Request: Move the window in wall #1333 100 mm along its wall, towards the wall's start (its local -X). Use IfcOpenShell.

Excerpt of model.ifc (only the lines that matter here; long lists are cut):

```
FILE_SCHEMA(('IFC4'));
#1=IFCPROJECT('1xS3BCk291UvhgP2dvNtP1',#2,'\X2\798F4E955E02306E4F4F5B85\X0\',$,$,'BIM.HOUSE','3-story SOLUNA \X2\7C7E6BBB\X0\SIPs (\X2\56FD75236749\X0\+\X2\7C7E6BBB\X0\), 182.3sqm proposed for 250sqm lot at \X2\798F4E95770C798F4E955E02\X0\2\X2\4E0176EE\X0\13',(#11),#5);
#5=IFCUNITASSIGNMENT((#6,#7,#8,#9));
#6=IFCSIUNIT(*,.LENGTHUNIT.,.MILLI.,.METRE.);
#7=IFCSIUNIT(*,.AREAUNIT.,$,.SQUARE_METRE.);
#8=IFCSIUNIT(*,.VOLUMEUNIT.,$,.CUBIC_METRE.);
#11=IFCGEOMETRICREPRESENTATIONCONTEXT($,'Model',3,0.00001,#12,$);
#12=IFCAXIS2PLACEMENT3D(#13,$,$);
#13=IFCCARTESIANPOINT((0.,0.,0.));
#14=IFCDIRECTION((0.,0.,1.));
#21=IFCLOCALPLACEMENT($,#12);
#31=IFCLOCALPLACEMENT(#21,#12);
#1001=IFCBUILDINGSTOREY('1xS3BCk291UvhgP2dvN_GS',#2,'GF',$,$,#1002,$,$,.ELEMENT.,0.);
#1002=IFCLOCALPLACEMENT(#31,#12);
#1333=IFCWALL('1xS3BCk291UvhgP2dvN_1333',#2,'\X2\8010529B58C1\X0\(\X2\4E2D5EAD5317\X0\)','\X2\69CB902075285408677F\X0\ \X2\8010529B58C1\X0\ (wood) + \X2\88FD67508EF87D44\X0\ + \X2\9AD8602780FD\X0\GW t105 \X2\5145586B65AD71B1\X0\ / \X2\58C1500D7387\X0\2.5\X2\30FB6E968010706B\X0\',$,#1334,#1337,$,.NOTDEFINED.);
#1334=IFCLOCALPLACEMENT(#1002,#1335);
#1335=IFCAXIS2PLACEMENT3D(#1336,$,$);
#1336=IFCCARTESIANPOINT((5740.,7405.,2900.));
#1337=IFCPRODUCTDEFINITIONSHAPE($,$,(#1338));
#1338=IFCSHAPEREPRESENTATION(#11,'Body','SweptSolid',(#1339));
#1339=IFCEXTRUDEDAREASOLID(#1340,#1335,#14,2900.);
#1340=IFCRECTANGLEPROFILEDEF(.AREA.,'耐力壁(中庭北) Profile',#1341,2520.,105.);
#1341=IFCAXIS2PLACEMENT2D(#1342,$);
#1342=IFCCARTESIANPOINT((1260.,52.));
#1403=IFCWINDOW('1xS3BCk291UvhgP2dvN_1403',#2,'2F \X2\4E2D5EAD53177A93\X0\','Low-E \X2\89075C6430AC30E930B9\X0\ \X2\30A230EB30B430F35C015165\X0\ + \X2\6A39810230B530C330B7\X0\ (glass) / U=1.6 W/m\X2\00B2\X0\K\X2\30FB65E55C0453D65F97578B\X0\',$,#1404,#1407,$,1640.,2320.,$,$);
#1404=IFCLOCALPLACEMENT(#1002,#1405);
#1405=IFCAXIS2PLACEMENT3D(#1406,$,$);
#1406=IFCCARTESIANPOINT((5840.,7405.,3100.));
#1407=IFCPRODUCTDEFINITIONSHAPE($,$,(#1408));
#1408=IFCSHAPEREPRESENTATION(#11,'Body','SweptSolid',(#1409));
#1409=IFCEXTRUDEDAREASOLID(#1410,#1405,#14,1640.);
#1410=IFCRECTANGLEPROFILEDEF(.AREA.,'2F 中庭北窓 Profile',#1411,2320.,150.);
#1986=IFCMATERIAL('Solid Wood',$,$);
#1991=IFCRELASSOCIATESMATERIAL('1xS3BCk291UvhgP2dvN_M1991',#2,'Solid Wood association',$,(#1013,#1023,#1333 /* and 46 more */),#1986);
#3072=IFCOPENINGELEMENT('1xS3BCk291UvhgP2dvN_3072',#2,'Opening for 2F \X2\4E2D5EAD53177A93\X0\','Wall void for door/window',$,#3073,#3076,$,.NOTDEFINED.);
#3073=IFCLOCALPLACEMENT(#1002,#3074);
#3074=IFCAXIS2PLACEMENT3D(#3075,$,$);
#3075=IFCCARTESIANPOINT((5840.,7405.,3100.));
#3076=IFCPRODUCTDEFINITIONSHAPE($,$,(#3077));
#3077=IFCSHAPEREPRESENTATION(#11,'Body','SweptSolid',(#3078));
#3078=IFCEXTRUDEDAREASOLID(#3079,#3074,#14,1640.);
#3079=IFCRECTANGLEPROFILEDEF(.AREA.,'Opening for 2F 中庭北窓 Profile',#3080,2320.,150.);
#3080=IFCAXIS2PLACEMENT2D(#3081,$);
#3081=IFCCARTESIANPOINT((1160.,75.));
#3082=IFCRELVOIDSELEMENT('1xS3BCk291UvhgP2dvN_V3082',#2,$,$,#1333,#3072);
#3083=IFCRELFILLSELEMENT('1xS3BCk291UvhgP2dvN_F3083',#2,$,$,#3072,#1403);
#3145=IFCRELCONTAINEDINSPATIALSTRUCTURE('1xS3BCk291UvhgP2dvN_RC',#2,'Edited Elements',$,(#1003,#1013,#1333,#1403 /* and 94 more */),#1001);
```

```python
import ifcopenshell
import ifcopenshell.api.geometry
import ifcopenshell.util.placement
import ifcopenshell.util.unit

model = ifcopenshell.open("model.ifc")
unit_scale = ifcopenshell.util.unit.calculate_unit_scale(model)

window = model.by_guid("1xS3BCk291UvhgP2dvN_1403")
opening = window.FillsVoids[0].RelatingOpeningElement
wall = opening.VoidsElements[0].RelatingBuildingElement

wall_matrix = ifcopenshell.util.placement.get_local_placement(wall.ObjectPlacement)
shift = wall_matrix[:3, 0] * -0.1 / unit_scale
before = ifcopenshell.util.placement.get_local_placement(window.ObjectPlacement)[:3, 3].copy()

# The window is not placed relative to its opening, so move both.
for product in (opening, window):
    matrix = ifcopenshell.util.placement.get_local_placement(product.ObjectPlacement)
    matrix[:3, 3] += shift
    ifcopenshell.api.geometry.edit_object_placement(model, product=product, matrix=matrix, is_si=False)

after = ifcopenshell.util.placement.get_local_placement(window.ObjectPlacement)[:3, 3]
print("window moved by", (after - before).round(3) + 0.0)

model.write("model_edited.ifc")
```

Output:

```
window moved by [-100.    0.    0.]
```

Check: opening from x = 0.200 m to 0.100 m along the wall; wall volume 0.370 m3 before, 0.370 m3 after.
